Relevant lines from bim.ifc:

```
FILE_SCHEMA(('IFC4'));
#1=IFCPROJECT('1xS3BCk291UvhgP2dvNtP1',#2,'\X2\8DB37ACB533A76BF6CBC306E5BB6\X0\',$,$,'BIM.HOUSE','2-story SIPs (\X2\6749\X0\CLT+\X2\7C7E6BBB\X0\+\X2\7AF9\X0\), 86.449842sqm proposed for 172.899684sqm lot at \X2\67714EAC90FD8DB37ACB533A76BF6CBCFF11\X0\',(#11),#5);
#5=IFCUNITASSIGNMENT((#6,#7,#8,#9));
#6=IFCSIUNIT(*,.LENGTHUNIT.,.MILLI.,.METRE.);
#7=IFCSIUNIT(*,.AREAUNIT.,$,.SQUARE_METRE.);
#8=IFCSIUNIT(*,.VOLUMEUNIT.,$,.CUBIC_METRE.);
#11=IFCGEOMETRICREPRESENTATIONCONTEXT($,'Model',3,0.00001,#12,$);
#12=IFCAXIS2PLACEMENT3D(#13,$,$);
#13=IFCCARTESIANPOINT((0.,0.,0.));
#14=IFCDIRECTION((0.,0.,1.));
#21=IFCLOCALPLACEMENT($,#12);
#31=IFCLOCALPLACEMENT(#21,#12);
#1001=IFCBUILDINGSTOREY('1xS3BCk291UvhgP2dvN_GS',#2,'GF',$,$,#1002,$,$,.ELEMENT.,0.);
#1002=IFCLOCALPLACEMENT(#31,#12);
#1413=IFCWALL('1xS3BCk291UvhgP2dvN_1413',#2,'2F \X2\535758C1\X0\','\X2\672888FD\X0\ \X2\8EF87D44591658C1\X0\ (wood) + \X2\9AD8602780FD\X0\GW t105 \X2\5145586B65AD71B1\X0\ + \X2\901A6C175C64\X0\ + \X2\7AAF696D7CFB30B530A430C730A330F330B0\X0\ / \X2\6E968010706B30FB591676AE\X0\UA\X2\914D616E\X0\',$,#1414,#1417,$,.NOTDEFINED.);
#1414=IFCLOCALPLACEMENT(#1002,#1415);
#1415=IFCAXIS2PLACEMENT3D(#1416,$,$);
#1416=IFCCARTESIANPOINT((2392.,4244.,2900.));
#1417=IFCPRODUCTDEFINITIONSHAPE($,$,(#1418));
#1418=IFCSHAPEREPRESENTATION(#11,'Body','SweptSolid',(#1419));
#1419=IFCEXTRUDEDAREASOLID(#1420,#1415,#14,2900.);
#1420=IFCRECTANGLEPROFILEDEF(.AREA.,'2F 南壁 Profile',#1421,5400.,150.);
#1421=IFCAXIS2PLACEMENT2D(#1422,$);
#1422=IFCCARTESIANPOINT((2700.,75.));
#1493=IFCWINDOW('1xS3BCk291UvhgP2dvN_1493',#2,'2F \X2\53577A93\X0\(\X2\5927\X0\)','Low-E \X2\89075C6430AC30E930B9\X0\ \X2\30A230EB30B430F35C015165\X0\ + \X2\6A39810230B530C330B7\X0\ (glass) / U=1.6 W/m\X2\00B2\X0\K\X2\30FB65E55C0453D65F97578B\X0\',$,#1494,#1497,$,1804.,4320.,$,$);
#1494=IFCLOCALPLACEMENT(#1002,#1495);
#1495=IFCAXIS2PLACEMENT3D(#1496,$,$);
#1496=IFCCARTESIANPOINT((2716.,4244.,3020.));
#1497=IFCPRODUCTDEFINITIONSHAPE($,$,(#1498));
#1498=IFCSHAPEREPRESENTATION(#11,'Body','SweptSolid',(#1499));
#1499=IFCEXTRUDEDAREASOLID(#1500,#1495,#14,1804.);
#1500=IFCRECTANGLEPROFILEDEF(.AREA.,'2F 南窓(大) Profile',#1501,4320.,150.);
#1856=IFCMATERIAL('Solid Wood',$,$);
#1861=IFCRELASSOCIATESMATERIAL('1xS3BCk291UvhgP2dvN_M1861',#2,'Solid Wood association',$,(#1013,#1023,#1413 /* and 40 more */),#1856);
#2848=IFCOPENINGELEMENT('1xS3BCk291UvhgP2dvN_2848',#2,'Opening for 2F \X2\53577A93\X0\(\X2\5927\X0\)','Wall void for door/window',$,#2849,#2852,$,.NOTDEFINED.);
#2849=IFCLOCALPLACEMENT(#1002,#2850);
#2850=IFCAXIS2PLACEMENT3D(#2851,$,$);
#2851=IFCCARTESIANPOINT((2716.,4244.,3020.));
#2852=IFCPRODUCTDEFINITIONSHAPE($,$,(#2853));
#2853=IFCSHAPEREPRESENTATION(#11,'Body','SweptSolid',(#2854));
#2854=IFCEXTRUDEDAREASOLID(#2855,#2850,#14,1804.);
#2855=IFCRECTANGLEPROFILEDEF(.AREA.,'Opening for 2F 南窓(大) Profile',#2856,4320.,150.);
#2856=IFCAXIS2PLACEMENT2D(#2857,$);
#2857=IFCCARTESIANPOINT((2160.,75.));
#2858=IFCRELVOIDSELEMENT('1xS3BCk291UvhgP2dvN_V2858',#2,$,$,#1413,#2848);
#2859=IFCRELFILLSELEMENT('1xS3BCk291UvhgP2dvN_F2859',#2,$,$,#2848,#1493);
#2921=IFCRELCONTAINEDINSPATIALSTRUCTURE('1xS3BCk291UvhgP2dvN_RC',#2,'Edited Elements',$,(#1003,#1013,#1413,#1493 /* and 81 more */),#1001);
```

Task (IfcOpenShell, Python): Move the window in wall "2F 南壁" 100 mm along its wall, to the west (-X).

```python
import ifcopenshell
import ifcopenshell.api.geometry
import ifcopenshell.util.placement

model = ifcopenshell.open("bim.ifc")

window = model.by_guid("1xS3BCk291UvhgP2dvN_1493")
opening = window.FillsVoids[0].RelatingOpeningElement
wall = opening.VoidsElements[0].RelatingBuildingElement

wall_matrix = ifcopenshell.util.placement.get_local_placement(wall.ObjectPlacement)
shift = wall_matrix[:3, 0] * -100.0
before = ifcopenshell.util.placement.get_local_placement(window.ObjectPlacement)[:3, 3].copy()

# The window is not placed relative to its opening, so move both.
for product in (opening, window):
    matrix = ifcopenshell.util.placement.get_local_placement(product.ObjectPlacement)
    matrix[:3, 3] += shift
    ifcopenshell.api.geometry.edit_object_placement(model, product=product, matrix=matrix, is_si=False)

after = ifcopenshell.util.placement.get_local_placement(window.ObjectPlacement)[:3, 3]
print("window moved by", (after - before).round(3) + 0.0)

model.write("bim_v2.ifc")
```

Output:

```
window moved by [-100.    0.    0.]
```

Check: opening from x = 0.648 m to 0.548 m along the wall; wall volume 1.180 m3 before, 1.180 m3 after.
